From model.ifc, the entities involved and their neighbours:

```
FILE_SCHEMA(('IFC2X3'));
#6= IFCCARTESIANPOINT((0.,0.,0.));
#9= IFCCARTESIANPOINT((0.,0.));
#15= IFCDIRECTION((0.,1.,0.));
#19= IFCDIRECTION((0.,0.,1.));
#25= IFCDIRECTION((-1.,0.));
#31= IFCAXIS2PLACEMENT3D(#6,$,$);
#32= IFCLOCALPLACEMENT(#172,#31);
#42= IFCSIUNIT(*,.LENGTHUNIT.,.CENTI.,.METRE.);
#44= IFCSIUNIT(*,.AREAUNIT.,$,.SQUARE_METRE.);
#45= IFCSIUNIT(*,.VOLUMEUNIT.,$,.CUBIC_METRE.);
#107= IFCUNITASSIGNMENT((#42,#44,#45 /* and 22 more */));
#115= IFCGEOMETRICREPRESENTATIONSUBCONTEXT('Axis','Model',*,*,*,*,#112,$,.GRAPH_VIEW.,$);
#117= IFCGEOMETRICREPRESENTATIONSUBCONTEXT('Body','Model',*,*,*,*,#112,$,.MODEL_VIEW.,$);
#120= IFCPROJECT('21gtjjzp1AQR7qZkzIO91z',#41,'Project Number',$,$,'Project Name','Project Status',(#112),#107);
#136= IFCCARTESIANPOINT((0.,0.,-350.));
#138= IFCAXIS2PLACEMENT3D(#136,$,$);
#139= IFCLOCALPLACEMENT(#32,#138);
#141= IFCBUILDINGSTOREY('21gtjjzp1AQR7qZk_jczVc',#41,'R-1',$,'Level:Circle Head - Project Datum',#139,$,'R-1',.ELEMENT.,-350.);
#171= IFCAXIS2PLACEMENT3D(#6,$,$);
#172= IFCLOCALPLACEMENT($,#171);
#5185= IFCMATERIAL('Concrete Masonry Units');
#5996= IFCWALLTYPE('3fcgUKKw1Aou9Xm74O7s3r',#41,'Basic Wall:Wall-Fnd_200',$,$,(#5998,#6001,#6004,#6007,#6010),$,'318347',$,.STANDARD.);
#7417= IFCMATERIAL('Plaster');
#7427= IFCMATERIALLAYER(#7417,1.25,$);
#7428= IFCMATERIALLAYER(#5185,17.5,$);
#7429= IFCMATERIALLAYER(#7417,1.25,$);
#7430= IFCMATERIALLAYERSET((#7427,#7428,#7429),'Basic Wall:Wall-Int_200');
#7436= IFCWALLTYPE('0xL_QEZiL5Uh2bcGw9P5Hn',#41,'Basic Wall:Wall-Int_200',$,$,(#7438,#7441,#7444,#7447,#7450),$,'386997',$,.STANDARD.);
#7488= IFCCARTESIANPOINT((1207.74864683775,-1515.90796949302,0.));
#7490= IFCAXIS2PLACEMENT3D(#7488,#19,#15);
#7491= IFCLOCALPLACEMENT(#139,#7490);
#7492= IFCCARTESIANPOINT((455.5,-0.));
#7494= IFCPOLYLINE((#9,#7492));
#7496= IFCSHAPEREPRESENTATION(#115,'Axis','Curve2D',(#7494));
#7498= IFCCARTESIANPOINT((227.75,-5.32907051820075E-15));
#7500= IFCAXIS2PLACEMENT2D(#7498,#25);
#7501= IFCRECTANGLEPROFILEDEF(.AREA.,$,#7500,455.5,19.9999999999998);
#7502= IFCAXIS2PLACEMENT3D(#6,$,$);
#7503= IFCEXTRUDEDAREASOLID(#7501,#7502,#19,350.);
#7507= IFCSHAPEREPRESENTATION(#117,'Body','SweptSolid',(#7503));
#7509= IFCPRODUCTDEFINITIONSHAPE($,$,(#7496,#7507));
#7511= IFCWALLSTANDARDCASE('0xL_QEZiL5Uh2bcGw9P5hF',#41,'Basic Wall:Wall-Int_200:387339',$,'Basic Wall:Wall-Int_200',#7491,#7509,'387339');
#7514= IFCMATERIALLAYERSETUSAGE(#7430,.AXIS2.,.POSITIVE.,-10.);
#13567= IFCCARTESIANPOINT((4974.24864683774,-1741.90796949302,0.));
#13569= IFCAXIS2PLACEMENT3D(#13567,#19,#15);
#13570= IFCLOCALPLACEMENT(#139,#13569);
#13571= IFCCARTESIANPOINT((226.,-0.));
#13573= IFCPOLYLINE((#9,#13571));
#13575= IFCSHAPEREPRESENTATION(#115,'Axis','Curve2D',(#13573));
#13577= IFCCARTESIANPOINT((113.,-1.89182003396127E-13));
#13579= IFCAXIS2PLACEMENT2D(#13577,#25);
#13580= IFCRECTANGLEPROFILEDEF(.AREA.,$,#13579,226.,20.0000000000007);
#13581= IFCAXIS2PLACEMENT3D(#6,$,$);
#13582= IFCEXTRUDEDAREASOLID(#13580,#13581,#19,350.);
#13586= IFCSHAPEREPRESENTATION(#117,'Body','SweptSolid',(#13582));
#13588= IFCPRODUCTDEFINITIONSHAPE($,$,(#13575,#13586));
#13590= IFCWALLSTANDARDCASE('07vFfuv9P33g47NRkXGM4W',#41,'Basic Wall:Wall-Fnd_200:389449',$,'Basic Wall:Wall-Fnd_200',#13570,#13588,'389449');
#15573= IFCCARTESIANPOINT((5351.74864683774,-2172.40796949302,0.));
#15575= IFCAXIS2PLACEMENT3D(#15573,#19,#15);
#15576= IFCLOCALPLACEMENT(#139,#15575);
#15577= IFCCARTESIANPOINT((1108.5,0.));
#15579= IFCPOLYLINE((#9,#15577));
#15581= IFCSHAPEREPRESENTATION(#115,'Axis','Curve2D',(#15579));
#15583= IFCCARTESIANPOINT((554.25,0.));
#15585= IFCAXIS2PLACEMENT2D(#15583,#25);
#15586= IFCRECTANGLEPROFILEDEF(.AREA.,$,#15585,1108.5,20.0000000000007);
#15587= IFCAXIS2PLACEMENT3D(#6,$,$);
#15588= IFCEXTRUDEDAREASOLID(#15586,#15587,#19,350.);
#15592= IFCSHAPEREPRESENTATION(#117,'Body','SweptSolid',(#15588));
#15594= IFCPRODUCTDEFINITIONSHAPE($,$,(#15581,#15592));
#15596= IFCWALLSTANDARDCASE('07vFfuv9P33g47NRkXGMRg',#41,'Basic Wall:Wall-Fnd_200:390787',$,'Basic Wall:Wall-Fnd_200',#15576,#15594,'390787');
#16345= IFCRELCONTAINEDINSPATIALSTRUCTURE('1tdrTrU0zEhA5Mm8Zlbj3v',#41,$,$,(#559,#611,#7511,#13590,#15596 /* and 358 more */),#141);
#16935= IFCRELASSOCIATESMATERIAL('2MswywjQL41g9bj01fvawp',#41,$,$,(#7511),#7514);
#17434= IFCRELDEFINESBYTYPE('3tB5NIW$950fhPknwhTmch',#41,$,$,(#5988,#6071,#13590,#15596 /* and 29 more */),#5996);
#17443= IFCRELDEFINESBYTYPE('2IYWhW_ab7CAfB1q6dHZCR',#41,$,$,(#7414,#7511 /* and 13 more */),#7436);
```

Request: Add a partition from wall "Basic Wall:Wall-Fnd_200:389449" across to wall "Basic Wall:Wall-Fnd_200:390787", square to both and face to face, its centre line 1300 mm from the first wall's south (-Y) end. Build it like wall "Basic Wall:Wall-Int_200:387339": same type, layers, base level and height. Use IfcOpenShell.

```python
import numpy as np
import ifcopenshell
import ifcopenshell.api.geometry
import ifcopenshell.api.material
import ifcopenshell.api.pset
import ifcopenshell.api.root
import ifcopenshell.api.spatial
import ifcopenshell.api.type
import ifcopenshell.geom
import ifcopenshell.util.element
import ifcopenshell.util.placement
import ifcopenshell.util.representation
import ifcopenshell.util.shape
import ifcopenshell.util.unit

model = ifcopenshell.open("model.ifc")
unit_scale = ifcopenshell.util.unit.calculate_unit_scale(model)
settings = ifcopenshell.geom.settings()
settings.set("use-world-coords", True)

start_wall = model.by_id(13590)
end_wall = model.by_guid("07vFfuv9P33g47NRkXGMRg")
like = model.by_guid("0xL_QEZiL5Uh2bcGw9P5hF")
matrix = ifcopenshell.util.placement.get_local_placement(start_wall.ObjectPlacement)
matrix[:3, 3] *= unit_scale


def extent(element):
    """Bounding box in the first wall's axes, in metres."""
    shape = ifcopenshell.geom.create_shape(settings, element)
    points = (ifcopenshell.util.shape.get_vertices(shape.geometry) - matrix[:3, 3]) @ matrix[:3, :3]
    return points.min(axis=0), points.max(axis=0)


y_start = extent(start_wall)[0][1]
y_end = extent(end_wall)[1][1]
like_min, like_max = extent(like)
length, height = float(abs(y_end - y_start)), float(like_max[2] - like_min[2])
layer_set = ifcopenshell.util.element.get_material(like, should_skip_usage=True)
thickness = sum(layer.LayerThickness for layer in layer_set.MaterialLayers) * unit_scale

wall = ifcopenshell.api.root.create_entity(model, ifc_class="IfcWallStandardCase", name="New partition")
storey = ifcopenshell.util.element.get_container(like)
ifcopenshell.api.spatial.assign_container(model, products=[wall], relating_structure=storey)
ifcopenshell.api.type.assign_type(
    model, related_objects=[wall], relating_type=ifcopenshell.util.element.get_type(like), should_map_representations=False
)
rel = ifcopenshell.api.material.assign_material(
    model, products=[wall], type="IfcMaterialLayerSetUsage", material=layer_set
)
rel.RelatingMaterial.OffsetFromReferenceLine = -thickness / 2 / unit_scale
pset = ifcopenshell.api.pset.add_pset(model, product=wall, name="Pset_WallCommon")
ifcopenshell.api.pset.edit_pset(model, pset=pset, properties={"IsExternal": False, "LoadBearing": False})

# The axis runs down the middle of the wall.
axis = ifcopenshell.api.geometry.add_axis_representation(
    model, context=ifcopenshell.util.representation.get_context(model, "Model", "Axis"), axis=[(0.0, 0.0), (length, 0.0)]
)
body = ifcopenshell.api.geometry.add_wall_representation(
    model,
    context=ifcopenshell.util.representation.get_context(model, "Model", "Body", "MODEL_VIEW"),
    length=length,
    height=height,
    thickness=thickness,
    offset=-thickness / 2,
)
for representation in (axis, body):
    ifcopenshell.api.geometry.assign_representation(model, product=wall, representation=representation)

placement = matrix @ ifcopenshell.util.placement.rotation(-90, "Z")
placement[:, 3] = matrix @ np.array([extent(start_wall)[0][0] + 1.3, y_start, like_min[2], 1.0])
ifcopenshell.api.geometry.edit_object_placement(model, product=wall, matrix=placement)

print(f"partition {length:.3f} m long, {height:.3f} m high, {thickness:.3f} m thick")

model.write("model_updated.ifc")
```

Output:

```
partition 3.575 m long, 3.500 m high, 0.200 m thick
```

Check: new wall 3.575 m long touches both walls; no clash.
